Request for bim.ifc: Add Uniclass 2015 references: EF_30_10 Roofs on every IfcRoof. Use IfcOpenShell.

First a look at what the model holds.

```python
import ifcopenshell

model = ifcopenshell.open("bim.ifc")
print(model.schema)
print("classifications:", [c.Name for c in model.by_type("IfcClassification")])
for ifc_class in ("IfcDoor", "IfcRoof", "IfcStair", "IfcWall", "IfcWindow"):
    print(ifc_class, len(model.by_type(ifc_class)))
```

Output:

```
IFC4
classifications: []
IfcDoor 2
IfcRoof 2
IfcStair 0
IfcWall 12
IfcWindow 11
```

```python
import ifcopenshell
import ifcopenshell.api.classification

model = ifcopenshell.open("bim.ifc")

system = ifcopenshell.api.classification.add_classification(model, classification="Uniclass 2015")

codes = {
    "IfcRoof": ("EF_30_10", "Roofs"),
}
for ifc_class, (code, name) in codes.items():
    products = model.by_type(ifc_class)
    ifcopenshell.api.classification.add_reference(
        model, products=products, classification=system, identification=code, name=name
    )
    print(code, len(products))

model.write("bim-out.ifc")
```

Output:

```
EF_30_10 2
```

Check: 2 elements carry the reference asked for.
